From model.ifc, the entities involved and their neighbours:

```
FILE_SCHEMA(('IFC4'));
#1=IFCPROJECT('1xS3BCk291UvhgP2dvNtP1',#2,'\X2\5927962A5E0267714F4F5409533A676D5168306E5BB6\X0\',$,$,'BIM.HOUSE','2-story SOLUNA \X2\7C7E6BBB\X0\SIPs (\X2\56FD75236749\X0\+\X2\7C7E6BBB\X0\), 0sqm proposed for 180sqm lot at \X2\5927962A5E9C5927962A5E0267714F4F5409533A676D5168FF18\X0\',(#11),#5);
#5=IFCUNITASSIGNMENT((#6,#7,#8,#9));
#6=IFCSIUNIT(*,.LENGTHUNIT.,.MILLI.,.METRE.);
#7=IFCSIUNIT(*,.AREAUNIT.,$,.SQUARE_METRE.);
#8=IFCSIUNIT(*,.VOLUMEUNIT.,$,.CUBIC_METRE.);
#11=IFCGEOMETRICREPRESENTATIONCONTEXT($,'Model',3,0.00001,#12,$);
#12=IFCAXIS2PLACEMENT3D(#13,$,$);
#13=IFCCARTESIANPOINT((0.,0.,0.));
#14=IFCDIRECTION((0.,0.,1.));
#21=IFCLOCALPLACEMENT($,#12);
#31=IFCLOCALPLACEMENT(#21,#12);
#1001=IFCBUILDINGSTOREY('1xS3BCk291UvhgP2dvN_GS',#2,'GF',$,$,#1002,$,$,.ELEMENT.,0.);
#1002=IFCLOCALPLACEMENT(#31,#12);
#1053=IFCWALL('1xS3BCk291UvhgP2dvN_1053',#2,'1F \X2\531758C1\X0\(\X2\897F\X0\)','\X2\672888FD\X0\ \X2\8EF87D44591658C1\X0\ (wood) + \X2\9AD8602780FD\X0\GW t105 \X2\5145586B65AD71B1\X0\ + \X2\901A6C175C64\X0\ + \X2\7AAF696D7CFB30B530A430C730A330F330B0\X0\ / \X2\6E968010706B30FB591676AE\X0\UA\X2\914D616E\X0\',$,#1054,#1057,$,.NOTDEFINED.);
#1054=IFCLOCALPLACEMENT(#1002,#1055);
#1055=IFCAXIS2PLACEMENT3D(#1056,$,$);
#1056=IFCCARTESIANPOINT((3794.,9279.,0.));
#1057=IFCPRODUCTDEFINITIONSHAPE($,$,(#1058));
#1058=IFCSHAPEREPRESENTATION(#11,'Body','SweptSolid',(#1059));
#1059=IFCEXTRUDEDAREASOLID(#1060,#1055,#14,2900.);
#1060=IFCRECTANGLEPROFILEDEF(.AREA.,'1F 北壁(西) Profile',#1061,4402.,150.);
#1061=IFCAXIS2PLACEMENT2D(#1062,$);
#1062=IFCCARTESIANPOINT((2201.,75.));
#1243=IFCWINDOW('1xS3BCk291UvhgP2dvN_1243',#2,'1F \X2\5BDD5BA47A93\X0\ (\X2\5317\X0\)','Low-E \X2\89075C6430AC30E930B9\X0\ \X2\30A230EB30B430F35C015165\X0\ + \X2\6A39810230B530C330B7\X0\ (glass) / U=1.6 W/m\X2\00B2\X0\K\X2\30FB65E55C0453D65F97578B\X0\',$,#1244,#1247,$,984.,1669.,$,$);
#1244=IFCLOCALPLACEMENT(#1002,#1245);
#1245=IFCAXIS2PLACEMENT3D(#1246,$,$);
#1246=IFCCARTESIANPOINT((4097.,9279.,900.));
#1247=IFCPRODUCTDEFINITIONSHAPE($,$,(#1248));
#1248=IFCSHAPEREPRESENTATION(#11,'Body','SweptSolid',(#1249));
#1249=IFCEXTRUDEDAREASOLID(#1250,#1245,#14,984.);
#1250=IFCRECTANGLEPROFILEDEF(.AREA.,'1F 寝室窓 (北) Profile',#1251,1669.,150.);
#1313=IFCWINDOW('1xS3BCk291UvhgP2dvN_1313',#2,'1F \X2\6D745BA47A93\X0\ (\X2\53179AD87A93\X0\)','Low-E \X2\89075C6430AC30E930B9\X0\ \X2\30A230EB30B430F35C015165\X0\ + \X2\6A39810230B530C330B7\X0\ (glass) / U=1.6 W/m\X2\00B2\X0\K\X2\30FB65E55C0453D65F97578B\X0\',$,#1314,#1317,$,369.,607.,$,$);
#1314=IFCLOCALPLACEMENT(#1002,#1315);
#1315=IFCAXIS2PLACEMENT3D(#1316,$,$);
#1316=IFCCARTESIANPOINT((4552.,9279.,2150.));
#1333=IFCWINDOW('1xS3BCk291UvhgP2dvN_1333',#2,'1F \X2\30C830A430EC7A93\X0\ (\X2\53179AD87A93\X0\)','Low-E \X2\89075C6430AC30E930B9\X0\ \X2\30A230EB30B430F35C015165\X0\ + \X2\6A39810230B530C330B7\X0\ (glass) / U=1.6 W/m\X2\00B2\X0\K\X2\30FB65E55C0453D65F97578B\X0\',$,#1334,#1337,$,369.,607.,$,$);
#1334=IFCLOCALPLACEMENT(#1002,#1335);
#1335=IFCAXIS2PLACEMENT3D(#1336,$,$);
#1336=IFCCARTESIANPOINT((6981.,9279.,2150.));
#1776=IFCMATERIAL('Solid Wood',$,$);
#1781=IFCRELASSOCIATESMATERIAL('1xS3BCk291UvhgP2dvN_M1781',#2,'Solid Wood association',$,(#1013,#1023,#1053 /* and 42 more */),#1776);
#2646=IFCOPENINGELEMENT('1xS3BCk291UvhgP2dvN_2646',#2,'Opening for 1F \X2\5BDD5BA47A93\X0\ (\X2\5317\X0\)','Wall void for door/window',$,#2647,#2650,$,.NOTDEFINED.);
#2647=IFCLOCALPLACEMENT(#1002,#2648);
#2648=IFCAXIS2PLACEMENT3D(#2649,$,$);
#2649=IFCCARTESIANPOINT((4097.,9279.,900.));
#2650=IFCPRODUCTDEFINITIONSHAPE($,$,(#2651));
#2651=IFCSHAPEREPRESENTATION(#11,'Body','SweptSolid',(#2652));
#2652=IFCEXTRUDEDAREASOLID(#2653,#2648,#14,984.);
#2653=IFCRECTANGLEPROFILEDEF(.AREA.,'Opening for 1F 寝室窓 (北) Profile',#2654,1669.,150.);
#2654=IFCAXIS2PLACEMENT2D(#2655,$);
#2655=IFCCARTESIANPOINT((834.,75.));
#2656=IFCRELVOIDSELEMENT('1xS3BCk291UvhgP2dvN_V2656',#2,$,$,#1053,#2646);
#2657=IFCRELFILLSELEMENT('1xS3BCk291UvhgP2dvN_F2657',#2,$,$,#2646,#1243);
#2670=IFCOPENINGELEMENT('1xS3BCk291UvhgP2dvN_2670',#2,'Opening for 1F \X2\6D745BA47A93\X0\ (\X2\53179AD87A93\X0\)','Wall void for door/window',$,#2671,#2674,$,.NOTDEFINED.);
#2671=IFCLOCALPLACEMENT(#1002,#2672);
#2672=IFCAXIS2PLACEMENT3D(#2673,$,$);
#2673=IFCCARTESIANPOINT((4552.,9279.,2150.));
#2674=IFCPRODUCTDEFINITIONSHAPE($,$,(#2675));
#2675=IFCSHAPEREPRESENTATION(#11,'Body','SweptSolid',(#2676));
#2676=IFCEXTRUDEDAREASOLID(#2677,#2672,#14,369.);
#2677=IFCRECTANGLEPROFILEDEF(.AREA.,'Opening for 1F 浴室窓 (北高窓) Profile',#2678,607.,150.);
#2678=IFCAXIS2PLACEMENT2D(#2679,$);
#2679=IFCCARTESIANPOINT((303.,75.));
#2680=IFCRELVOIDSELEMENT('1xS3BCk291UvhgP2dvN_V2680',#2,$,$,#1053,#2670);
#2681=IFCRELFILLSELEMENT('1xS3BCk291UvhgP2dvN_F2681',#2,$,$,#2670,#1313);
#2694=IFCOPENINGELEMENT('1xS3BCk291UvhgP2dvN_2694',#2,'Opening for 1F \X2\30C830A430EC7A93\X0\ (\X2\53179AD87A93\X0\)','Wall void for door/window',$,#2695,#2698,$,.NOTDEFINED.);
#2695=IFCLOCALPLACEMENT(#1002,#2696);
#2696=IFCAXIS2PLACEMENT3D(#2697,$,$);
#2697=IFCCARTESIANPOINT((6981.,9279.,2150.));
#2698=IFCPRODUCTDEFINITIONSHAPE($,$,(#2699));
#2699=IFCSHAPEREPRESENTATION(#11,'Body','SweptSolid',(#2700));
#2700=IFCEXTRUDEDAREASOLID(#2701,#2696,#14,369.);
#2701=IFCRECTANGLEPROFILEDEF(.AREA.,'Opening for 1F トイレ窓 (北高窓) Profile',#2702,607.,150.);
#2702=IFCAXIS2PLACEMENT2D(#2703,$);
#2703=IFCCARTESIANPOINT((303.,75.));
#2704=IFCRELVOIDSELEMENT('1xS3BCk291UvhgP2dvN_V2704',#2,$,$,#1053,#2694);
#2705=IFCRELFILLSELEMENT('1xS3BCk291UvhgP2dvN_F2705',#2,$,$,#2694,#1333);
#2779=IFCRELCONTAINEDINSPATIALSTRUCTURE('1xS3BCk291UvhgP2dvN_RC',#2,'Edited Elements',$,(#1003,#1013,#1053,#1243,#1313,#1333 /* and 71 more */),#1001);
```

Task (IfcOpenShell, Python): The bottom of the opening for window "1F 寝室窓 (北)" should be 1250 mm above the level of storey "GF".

```python
import numpy as np
import ifcopenshell
import ifcopenshell.api.geometry
import ifcopenshell.geom
import ifcopenshell.util.element
import ifcopenshell.util.placement
import ifcopenshell.util.shape
import ifcopenshell.util.unit

model = ifcopenshell.open("model.ifc")
unit_scale = ifcopenshell.util.unit.calculate_unit_scale(model)

window = model.by_guid("1xS3BCk291UvhgP2dvN_1243")
opening = window.FillsVoids[0].RelatingOpeningElement
storey = ifcopenshell.util.element.get_container(window, ifc_class="IfcBuildingStorey")
level = ifcopenshell.util.placement.get_local_placement(storey.ObjectPlacement)[2, 3]

# The opening's origin need not be at the sill, so measure its lowest point.
shape = ifcopenshell.geom.create_shape(ifcopenshell.geom.settings(), opening)
bottom = ifcopenshell.util.shape.get_shape_bottom_elevation(shape, shape.geometry) / unit_scale
dz = level + 1.25 / unit_scale - bottom

shift = np.array([0.0, 0.0, dz])
# The window is not placed relative to its opening, so move both.
for product in (opening, window):
    matrix = ifcopenshell.util.placement.get_local_placement(product.ObjectPlacement)
    matrix[:3, 3] += shift
    ifcopenshell.api.geometry.edit_object_placement(model, product=product, matrix=matrix, is_si=False)

print(f"moved by {dz * unit_scale:+.3f} m")

model.write("model_v2.ifc")
```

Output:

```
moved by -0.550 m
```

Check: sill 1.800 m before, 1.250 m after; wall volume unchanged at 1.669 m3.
